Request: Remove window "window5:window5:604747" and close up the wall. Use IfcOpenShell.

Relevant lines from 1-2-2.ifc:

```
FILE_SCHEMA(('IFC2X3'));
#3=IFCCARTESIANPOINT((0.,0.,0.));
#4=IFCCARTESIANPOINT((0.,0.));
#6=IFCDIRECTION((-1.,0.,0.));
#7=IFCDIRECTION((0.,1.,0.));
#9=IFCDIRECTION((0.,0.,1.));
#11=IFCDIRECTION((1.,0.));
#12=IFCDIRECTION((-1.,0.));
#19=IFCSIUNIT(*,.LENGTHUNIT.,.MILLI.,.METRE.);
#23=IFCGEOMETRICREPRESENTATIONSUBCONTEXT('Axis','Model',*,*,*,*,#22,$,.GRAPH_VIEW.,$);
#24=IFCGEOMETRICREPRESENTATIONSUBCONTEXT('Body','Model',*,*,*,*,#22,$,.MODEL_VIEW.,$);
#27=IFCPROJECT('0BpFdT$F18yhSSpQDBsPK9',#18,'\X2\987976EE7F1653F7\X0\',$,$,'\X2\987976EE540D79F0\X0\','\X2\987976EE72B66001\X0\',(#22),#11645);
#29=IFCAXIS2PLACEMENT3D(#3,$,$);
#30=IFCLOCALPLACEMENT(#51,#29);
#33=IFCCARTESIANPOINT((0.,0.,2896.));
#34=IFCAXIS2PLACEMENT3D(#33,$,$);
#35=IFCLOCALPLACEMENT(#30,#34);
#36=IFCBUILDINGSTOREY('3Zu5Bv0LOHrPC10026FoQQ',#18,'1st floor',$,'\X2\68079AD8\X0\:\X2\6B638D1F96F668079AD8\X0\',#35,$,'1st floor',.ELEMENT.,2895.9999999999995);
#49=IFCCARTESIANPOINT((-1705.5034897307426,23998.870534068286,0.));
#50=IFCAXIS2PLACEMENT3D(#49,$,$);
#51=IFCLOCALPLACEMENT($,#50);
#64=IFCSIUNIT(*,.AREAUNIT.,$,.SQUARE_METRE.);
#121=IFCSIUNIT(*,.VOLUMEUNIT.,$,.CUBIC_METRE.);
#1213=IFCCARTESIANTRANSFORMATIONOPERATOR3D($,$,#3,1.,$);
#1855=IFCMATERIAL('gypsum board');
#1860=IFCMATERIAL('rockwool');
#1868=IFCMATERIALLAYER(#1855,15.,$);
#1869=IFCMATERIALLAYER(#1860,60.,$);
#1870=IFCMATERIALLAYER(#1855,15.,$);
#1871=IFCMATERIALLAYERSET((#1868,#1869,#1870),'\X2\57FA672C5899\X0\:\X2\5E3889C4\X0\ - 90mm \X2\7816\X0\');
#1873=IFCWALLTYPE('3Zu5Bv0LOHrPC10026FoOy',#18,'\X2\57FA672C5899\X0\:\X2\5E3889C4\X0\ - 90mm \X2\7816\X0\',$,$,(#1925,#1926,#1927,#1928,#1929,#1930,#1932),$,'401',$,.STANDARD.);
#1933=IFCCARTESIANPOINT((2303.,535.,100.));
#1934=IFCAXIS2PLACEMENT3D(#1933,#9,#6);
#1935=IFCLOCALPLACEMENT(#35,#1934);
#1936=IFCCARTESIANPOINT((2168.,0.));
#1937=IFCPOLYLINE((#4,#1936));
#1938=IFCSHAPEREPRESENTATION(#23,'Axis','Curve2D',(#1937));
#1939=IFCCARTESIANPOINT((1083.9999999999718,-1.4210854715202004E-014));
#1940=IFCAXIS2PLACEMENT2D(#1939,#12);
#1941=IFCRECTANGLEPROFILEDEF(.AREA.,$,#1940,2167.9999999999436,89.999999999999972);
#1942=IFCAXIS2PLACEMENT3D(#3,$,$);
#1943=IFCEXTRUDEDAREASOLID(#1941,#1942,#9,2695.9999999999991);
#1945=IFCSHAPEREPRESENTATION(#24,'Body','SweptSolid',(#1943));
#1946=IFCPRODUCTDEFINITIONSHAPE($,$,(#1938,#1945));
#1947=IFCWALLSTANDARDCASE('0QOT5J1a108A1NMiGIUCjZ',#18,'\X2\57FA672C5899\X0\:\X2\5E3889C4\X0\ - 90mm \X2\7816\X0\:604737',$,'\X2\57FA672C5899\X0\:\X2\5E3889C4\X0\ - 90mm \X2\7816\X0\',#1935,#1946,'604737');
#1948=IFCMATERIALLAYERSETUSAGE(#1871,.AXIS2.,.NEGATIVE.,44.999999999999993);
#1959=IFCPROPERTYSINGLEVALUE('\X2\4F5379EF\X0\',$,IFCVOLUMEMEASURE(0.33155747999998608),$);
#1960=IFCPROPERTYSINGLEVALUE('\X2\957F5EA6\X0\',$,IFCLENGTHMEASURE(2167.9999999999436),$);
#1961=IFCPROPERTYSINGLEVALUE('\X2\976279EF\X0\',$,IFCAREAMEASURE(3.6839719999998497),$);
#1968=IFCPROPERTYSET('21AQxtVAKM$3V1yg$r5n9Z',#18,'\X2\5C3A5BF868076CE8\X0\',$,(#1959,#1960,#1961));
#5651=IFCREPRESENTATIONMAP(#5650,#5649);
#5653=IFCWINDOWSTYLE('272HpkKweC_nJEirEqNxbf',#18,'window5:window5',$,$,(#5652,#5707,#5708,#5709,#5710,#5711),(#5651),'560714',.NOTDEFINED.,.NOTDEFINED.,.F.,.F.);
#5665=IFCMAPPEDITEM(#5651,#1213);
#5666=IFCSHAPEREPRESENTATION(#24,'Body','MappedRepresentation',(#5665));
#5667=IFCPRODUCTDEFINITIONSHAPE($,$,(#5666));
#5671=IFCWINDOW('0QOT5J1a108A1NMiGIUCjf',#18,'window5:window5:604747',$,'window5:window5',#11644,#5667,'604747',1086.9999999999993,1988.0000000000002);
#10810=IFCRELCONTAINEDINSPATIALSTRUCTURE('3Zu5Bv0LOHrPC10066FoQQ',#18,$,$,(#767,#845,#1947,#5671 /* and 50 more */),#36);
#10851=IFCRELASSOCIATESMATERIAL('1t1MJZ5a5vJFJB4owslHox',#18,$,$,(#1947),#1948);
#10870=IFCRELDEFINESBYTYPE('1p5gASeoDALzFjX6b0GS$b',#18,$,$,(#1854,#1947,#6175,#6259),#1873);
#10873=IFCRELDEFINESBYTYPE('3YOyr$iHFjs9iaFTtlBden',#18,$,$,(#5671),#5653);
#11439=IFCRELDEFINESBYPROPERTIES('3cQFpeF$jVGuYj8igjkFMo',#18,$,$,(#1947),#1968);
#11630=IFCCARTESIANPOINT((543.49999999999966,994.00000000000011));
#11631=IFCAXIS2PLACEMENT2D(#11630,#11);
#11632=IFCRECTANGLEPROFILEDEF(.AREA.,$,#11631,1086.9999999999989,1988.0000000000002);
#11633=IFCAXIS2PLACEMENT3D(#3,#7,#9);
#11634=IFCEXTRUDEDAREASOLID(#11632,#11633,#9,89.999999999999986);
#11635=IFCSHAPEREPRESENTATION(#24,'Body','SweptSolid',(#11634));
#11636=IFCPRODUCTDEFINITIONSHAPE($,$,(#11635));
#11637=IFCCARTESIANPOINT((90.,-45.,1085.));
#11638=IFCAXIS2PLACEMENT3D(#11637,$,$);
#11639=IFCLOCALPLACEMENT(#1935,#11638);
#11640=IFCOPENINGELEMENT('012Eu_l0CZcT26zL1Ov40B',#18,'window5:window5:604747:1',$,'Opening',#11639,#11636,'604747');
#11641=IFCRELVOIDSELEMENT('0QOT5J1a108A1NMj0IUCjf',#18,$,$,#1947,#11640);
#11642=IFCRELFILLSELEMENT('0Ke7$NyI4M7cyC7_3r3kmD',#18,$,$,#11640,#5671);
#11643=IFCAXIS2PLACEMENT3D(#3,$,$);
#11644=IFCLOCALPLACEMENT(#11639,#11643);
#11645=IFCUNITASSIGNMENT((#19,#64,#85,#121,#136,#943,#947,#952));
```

```python
import ifcopenshell
import ifcopenshell.api.feature
import ifcopenshell.api.pset
import ifcopenshell.api.root
import ifcopenshell.geom
import ifcopenshell.util.element
import ifcopenshell.util.shape
import ifcopenshell.util.unit

model = ifcopenshell.open("1-2-2.ifc")
area_scale = ifcopenshell.util.unit.calculate_unit_scale(model, "AREAUNIT")
volume_scale = ifcopenshell.util.unit.calculate_unit_scale(model, "VOLUMEUNIT")
settings = ifcopenshell.geom.settings()


def volume(element):
    """Net volume in cubic metres, openings subtracted."""
    shape = ifcopenshell.geom.create_shape(settings, element)
    return ifcopenshell.util.shape.get_volume(shape.geometry)


window = model.by_id(5671)
opening = window.FillsVoids[0].RelatingOpeningElement
wall = opening.VoidsElements[0].RelatingBuildingElement
before = volume(wall)

ifcopenshell.api.root.remove_product(model, product=window)
ifcopenshell.api.feature.remove_feature(model, feature=opening)

after = volume(wall)
thickness = 0.09  # wall thickness in metres

# Update the wall's stored quantities.
pset = model.by_id(ifcopenshell.util.element.get_pset(wall, "尺寸标注", should_inherit=False)["id"])
ifcopenshell.api.pset.edit_pset(model, pset=pset, properties={
    "体积": model.create_entity("IfcVolumeMeasure", after / volume_scale),
    "面积": model.create_entity("IfcAreaMeasure", after / thickness / area_scale),
})

print(f"wall volume {before:.3f} -> {after:.3f} m3")

model.write("1-2-2_rev.ifc")
```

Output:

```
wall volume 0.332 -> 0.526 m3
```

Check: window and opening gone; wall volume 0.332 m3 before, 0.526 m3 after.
